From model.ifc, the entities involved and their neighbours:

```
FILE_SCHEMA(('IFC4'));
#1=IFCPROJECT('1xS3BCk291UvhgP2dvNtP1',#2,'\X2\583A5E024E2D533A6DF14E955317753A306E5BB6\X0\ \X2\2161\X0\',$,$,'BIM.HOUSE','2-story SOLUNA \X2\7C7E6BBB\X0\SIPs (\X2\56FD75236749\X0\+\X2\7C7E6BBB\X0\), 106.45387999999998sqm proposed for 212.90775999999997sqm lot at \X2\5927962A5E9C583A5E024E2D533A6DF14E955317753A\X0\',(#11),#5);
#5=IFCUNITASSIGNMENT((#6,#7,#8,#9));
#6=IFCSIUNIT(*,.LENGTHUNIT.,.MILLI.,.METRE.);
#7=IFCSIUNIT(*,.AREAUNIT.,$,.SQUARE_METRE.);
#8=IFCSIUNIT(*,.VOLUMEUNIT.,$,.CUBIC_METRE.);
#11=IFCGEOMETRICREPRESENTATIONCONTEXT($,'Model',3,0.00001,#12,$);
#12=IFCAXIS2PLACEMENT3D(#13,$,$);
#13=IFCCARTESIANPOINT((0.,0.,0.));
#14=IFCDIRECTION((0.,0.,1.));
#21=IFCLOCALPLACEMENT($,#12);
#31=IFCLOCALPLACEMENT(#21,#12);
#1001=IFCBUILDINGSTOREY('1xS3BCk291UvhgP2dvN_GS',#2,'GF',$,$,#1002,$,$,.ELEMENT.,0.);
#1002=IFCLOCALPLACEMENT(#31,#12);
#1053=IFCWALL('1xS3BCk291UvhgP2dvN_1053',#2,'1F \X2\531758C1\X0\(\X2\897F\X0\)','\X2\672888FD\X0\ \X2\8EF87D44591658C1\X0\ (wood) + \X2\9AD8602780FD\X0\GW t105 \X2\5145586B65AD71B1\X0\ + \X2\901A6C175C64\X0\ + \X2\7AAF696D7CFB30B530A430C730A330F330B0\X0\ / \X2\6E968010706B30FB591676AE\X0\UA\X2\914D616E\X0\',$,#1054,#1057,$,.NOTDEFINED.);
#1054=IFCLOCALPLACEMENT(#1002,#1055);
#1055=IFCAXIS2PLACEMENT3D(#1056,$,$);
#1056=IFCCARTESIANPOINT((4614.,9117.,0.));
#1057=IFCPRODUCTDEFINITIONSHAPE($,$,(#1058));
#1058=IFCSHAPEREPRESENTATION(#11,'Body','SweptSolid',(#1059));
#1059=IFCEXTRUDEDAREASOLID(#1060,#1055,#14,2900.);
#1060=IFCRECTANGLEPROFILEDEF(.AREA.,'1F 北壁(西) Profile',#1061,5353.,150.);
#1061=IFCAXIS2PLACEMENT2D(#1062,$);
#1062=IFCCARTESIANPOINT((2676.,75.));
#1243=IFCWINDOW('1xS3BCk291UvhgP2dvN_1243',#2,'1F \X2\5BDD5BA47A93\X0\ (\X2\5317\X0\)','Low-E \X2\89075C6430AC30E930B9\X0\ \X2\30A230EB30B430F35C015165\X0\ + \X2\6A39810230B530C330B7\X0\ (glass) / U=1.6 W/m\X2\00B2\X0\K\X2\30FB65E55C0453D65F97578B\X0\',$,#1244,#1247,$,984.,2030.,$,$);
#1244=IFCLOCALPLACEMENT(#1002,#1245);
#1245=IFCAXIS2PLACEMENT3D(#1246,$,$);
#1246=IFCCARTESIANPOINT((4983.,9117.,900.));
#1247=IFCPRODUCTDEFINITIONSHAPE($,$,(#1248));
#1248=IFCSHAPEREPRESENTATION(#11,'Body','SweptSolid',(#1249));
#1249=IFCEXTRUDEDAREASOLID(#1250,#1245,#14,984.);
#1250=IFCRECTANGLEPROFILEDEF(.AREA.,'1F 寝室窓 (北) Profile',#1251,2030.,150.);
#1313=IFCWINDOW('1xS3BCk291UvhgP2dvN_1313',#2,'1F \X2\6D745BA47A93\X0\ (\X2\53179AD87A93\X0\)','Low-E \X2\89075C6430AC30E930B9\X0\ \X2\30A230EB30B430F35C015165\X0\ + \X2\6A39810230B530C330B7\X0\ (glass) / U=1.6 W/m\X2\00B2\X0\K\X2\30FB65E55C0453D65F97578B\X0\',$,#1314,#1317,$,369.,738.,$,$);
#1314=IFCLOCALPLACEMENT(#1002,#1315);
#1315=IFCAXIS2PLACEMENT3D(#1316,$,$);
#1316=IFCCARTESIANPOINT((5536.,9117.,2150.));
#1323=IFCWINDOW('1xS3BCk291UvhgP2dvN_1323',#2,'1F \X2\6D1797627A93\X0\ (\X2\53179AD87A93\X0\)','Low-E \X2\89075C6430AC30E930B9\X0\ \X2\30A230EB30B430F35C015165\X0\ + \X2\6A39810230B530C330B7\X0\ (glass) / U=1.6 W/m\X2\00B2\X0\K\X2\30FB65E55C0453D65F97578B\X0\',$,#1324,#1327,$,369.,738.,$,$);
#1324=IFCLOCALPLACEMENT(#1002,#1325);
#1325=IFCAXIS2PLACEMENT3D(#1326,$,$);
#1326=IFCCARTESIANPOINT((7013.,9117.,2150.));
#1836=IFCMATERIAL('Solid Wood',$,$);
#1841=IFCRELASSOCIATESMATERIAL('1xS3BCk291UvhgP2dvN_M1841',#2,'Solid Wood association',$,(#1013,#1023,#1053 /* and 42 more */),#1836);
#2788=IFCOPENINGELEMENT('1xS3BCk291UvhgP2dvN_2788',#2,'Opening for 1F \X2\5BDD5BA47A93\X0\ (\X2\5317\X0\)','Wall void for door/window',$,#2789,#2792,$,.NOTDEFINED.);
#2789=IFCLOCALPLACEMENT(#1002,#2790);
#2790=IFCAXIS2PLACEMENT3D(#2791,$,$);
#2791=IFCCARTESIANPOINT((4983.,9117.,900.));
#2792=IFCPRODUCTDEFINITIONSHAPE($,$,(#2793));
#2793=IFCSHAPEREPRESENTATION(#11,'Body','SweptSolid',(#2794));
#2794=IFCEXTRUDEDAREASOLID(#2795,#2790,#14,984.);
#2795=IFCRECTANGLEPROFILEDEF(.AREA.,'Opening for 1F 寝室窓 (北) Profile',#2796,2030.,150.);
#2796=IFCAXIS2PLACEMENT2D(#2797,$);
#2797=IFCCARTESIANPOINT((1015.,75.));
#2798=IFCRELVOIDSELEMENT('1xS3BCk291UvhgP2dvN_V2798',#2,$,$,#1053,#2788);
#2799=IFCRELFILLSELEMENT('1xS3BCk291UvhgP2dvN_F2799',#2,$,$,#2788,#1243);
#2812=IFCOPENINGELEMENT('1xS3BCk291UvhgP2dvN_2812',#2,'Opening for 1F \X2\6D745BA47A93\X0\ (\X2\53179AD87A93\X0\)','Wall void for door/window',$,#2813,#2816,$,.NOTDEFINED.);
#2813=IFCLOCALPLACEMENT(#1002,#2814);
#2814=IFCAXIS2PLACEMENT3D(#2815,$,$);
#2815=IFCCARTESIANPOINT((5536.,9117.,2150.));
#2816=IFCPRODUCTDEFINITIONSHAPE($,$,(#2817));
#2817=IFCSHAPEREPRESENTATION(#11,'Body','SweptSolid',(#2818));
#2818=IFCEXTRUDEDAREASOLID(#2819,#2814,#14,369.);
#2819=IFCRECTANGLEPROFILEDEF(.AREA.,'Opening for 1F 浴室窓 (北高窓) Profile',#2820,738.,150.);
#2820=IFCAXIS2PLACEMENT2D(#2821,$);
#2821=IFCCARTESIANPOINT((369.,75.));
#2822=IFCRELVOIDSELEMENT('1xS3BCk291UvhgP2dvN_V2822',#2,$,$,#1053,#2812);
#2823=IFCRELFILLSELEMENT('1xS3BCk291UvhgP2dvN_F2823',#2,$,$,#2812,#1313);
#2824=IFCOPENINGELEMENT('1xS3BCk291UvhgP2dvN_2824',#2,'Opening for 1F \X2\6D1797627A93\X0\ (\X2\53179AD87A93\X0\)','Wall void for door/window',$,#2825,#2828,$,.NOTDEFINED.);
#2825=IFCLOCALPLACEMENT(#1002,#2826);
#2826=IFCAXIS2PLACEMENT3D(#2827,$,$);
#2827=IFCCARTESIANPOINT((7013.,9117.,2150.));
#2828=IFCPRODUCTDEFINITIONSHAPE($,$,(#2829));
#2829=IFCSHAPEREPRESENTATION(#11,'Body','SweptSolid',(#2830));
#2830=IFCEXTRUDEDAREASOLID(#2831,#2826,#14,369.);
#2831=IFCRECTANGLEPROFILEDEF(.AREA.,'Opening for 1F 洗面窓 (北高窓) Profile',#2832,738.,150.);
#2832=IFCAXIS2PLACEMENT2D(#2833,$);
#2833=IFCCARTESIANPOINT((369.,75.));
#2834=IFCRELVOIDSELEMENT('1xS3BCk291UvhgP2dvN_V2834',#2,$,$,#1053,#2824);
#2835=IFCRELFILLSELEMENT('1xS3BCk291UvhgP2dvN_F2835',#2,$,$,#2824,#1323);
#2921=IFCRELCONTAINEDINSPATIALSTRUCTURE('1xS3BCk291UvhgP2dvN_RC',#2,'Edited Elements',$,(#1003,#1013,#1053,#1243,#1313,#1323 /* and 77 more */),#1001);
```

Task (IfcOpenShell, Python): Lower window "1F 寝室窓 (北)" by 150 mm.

```python
import numpy as np
import ifcopenshell
import ifcopenshell.api.geometry
import ifcopenshell.util.placement
import ifcopenshell.util.unit

model = ifcopenshell.open("model.ifc")
unit_scale = ifcopenshell.util.unit.calculate_unit_scale(model)

window = model.by_guid("1xS3BCk291UvhgP2dvN_1243")
opening = window.FillsVoids[0].RelatingOpeningElement
dz = -0.15 / unit_scale

shift = np.array([0.0, 0.0, dz])
# The window is not placed relative to its opening, so move both.
for product in (opening, window):
    matrix = ifcopenshell.util.placement.get_local_placement(product.ObjectPlacement)
    matrix[:3, 3] += shift
    ifcopenshell.api.geometry.edit_object_placement(model, product=product, matrix=matrix, is_si=False)

print(f"moved by {dz * unit_scale:+.3f} m")

model.write("model-out.ifc")
```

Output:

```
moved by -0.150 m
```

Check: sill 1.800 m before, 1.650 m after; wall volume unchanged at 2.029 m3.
